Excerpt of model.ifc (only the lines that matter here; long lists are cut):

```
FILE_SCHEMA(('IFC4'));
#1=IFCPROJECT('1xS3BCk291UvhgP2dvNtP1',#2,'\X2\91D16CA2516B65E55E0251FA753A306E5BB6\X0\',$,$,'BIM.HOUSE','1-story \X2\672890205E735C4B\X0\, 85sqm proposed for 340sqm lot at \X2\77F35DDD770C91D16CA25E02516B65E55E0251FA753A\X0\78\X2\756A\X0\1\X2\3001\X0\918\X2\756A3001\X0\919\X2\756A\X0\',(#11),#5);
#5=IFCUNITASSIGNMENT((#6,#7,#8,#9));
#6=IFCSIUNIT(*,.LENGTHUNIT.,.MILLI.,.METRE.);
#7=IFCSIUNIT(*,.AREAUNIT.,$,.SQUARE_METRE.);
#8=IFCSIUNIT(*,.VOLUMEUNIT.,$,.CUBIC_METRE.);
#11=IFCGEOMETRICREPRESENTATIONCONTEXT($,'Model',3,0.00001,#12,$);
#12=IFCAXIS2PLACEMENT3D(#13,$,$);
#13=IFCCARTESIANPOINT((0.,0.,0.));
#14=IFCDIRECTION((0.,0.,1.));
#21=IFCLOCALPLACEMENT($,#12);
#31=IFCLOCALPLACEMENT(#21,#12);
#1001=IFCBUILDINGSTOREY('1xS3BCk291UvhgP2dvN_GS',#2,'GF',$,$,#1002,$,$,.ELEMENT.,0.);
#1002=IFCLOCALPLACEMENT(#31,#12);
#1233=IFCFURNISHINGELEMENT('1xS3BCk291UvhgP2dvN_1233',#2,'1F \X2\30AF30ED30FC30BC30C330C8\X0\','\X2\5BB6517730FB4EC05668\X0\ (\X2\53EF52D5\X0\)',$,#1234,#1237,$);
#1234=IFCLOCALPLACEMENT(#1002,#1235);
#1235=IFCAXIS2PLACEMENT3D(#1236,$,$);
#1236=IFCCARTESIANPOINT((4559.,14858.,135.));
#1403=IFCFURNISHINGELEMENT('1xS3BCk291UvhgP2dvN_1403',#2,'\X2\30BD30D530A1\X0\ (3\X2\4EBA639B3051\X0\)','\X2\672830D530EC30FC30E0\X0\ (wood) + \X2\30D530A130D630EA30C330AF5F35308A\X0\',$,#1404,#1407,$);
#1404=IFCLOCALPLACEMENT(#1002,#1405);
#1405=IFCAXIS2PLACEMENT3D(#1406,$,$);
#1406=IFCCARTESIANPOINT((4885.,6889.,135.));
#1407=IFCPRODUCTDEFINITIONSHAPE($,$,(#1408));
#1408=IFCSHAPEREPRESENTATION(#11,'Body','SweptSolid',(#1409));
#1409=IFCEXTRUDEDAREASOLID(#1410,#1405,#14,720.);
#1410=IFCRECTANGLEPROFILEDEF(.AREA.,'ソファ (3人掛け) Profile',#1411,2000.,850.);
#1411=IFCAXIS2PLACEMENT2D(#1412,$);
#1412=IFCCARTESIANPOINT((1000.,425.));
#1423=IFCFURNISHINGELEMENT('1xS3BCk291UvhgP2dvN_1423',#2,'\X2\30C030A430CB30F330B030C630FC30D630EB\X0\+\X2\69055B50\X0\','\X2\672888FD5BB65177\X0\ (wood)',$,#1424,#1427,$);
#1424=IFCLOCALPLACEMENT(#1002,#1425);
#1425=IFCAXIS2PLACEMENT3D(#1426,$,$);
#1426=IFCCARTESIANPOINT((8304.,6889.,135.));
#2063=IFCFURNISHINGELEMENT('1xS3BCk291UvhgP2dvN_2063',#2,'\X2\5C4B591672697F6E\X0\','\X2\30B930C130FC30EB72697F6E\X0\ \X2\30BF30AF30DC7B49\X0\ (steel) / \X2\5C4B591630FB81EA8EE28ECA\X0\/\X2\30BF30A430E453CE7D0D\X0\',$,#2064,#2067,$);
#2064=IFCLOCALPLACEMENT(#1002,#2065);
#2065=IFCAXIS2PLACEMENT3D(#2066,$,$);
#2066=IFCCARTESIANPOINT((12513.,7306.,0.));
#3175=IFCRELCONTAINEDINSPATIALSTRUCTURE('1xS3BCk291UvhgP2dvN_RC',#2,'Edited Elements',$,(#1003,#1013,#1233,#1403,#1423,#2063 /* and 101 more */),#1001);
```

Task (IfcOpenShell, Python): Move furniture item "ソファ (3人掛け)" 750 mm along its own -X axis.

```python
import ifcopenshell
import ifcopenshell.api.geometry
import ifcopenshell.util.placement
import ifcopenshell.util.unit

model = ifcopenshell.open("model.ifc")
unit_scale = ifcopenshell.util.unit.calculate_unit_scale(model)

item = model.by_id(1403)
matrix = ifcopenshell.util.placement.get_local_placement(item.ObjectPlacement)
matrix[:3, 3] -= matrix[:3, 0] * 0.75 / unit_scale
ifcopenshell.api.geometry.edit_object_placement(model, product=item, matrix=matrix, is_si=False)

print(ifcopenshell.util.placement.get_local_placement(item.ObjectPlacement).round(3) + 0.0)

model.write("model-out.ifc")
```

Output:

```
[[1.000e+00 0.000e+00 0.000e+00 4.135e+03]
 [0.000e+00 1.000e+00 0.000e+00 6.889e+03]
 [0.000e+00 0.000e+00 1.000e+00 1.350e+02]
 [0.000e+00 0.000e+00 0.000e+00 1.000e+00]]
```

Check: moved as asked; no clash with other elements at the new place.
